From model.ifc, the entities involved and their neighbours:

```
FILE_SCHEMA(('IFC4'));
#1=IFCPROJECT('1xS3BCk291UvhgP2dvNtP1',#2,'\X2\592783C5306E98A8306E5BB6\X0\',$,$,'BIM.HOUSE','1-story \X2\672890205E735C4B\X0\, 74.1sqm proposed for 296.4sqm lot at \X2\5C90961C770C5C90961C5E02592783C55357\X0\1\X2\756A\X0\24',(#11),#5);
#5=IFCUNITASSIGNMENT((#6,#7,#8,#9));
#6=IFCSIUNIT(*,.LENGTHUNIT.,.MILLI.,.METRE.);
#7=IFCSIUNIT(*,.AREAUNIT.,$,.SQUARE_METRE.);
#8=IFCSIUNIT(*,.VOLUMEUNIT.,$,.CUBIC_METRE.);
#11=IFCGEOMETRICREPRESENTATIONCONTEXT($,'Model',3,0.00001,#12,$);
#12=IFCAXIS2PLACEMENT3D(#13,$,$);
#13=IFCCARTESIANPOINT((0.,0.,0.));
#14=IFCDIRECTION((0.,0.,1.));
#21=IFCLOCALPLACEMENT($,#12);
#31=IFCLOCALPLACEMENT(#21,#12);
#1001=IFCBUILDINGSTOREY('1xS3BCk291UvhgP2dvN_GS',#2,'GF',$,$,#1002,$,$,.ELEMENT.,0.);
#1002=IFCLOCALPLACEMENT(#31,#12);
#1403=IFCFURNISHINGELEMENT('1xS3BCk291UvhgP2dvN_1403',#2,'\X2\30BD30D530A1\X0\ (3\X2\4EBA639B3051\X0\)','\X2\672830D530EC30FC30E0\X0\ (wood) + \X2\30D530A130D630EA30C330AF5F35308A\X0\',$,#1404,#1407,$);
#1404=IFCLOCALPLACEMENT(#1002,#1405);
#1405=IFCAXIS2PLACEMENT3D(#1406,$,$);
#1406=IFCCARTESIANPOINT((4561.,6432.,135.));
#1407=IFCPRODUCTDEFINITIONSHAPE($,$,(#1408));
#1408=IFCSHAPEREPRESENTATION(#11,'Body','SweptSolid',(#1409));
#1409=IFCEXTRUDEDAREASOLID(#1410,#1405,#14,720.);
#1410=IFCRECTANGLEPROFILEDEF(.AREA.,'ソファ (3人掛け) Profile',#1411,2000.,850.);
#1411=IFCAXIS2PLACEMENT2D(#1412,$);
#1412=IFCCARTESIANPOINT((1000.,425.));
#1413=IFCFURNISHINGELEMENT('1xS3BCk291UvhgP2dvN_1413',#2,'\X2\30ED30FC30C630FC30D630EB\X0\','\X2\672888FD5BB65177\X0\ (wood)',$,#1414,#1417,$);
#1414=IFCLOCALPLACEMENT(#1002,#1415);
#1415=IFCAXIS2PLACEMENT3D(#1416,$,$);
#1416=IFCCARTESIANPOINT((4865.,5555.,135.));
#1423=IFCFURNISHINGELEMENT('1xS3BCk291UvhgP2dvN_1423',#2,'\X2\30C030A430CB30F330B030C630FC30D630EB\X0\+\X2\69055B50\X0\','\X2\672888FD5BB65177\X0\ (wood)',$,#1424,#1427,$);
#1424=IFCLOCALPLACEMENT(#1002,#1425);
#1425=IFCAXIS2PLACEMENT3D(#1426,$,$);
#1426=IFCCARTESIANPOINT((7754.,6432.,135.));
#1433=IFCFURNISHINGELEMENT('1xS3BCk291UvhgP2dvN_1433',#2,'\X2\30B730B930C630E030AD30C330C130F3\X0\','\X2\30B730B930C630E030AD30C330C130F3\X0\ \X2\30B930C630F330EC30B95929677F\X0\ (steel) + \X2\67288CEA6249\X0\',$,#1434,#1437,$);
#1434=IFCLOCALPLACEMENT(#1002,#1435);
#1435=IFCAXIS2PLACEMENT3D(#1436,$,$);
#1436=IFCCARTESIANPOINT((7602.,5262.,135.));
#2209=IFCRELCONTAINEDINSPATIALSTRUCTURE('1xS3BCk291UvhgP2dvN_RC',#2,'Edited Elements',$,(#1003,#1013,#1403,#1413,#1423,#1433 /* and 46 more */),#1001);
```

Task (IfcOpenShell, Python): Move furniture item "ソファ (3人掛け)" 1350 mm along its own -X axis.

```python
import ifcopenshell
import ifcopenshell.api.geometry
import ifcopenshell.util.placement

model = ifcopenshell.open("model.ifc")

item = model.by_id(1403)
matrix = ifcopenshell.util.placement.get_local_placement(item.ObjectPlacement)
matrix[:3, 3] -= matrix[:3, 0] * 1350.0
ifcopenshell.api.geometry.edit_object_placement(model, product=item, matrix=matrix, is_si=False)

print(ifcopenshell.util.placement.get_local_placement(item.ObjectPlacement).round(3) + 0.0)

model.write("model_updated.ifc")
```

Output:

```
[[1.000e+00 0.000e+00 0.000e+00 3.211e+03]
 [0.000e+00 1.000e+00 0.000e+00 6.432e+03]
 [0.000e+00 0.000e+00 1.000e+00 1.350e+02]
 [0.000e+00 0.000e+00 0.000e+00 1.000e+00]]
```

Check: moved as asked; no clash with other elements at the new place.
